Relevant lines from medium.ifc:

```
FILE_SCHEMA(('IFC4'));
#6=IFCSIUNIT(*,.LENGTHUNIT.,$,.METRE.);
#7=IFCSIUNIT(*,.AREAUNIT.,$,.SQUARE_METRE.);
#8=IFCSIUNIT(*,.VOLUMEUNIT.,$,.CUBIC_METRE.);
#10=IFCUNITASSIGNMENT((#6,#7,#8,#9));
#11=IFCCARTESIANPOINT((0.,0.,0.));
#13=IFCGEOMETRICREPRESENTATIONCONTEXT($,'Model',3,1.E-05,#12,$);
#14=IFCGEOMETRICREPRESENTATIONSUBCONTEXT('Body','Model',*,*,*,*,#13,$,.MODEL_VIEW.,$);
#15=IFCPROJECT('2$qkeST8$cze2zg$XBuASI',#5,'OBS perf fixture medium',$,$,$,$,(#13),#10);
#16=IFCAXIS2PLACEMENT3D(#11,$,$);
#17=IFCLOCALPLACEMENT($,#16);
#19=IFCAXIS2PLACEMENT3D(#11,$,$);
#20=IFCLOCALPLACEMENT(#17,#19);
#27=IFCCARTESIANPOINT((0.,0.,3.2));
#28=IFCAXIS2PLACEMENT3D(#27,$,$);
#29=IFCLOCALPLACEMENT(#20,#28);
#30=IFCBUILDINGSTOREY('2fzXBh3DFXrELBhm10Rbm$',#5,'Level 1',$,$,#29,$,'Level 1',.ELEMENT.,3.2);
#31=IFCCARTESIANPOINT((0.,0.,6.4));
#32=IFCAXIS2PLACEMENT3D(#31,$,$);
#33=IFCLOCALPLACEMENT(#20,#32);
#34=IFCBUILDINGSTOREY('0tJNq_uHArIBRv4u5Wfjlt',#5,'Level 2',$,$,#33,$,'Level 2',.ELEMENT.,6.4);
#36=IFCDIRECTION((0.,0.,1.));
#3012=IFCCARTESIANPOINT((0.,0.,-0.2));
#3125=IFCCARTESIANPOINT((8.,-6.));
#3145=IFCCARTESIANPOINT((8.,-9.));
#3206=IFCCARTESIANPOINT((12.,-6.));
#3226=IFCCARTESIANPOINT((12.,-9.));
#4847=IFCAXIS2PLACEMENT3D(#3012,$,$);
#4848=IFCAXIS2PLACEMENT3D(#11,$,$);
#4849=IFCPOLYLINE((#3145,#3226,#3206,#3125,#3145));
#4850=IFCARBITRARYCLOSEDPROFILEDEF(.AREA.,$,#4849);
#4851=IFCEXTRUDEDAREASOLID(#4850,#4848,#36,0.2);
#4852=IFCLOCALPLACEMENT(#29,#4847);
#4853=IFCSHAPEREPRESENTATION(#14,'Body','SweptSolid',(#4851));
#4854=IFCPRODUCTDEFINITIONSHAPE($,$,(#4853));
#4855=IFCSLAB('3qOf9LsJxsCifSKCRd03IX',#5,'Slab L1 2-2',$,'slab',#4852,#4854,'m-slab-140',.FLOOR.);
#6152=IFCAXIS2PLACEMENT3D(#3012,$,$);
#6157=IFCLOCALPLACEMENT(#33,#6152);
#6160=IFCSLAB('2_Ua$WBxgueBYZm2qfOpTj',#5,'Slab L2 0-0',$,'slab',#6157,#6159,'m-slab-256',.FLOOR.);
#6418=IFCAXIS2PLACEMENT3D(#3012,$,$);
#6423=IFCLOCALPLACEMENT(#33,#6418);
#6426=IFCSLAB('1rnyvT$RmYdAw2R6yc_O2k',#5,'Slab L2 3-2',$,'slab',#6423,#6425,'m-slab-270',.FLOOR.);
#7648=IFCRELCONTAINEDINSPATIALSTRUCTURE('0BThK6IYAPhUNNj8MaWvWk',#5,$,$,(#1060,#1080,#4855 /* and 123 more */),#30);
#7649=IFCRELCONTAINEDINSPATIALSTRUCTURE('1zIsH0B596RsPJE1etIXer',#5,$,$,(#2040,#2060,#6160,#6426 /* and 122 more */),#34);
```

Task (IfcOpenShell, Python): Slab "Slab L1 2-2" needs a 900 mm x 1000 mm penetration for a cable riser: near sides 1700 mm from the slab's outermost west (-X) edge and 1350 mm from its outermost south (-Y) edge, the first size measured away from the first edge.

```python
import numpy as np
import ifcopenshell
import ifcopenshell.api.feature
import ifcopenshell.api.geometry
import ifcopenshell.api.root
import ifcopenshell.geom
import ifcopenshell.util.placement
import ifcopenshell.util.representation
import ifcopenshell.util.shape
import ifcopenshell.util.unit

model = ifcopenshell.open("medium.ifc")
unit_scale = ifcopenshell.util.unit.calculate_unit_scale(model)
settings = ifcopenshell.geom.settings()


def volume(element):
    """Net volume in cubic metres, openings subtracted."""
    shape = ifcopenshell.geom.create_shape(settings, element)
    return ifcopenshell.util.shape.get_volume(shape.geometry)


slab = model.by_guid("3qOf9LsJxsCifSKCRd03IX")
before = volume(slab)

# Extent in the slab's own axes, in metres. The edges named are its -X and -Y sides.
slab_shape = ifcopenshell.geom.create_shape(settings, slab)
vertices = ifcopenshell.util.shape.get_vertices(slab_shape.geometry)
x_min, y_min, bottom = vertices.min(axis=0)
top = vertices[:, 2].max()

opening = ifcopenshell.api.root.create_entity(model, ifc_class="IfcOpeningElement", name="Cable riser opening", predefined_type="OPENING")
context = ifcopenshell.util.representation.get_context(model, "Model", "Body", "MODEL_VIEW")
width, depth = 0.9, 1
outline = [(0.0, 0.0), (width, 0.0), (width, depth), (0.0, depth), (0.0, 0.0)]
# Overshoot both faces by 50 mm so the cut is clean.
shape = ifcopenshell.api.geometry.add_slab_representation(
    model, context=context, depth=top - bottom + 0.1, polyline=outline
)
ifcopenshell.api.geometry.assign_representation(model, product=opening, representation=shape)

matrix = ifcopenshell.util.placement.get_local_placement(slab.ObjectPlacement)
matrix[:, 3] = matrix @ np.append(np.array([x_min + 1.7, y_min + 1.35, bottom - 0.05]) / unit_scale, 1.0)
ifcopenshell.api.geometry.edit_object_placement(model, product=opening, matrix=matrix, is_si=False)
ifcopenshell.api.feature.add_feature(model, feature=opening, element=slab)

after = volume(slab)

print(f"slab volume {before:.3f} -> {after:.3f} m3")

model.write("medium-out.ifc")
```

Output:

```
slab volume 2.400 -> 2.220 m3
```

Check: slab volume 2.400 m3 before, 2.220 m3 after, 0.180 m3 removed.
